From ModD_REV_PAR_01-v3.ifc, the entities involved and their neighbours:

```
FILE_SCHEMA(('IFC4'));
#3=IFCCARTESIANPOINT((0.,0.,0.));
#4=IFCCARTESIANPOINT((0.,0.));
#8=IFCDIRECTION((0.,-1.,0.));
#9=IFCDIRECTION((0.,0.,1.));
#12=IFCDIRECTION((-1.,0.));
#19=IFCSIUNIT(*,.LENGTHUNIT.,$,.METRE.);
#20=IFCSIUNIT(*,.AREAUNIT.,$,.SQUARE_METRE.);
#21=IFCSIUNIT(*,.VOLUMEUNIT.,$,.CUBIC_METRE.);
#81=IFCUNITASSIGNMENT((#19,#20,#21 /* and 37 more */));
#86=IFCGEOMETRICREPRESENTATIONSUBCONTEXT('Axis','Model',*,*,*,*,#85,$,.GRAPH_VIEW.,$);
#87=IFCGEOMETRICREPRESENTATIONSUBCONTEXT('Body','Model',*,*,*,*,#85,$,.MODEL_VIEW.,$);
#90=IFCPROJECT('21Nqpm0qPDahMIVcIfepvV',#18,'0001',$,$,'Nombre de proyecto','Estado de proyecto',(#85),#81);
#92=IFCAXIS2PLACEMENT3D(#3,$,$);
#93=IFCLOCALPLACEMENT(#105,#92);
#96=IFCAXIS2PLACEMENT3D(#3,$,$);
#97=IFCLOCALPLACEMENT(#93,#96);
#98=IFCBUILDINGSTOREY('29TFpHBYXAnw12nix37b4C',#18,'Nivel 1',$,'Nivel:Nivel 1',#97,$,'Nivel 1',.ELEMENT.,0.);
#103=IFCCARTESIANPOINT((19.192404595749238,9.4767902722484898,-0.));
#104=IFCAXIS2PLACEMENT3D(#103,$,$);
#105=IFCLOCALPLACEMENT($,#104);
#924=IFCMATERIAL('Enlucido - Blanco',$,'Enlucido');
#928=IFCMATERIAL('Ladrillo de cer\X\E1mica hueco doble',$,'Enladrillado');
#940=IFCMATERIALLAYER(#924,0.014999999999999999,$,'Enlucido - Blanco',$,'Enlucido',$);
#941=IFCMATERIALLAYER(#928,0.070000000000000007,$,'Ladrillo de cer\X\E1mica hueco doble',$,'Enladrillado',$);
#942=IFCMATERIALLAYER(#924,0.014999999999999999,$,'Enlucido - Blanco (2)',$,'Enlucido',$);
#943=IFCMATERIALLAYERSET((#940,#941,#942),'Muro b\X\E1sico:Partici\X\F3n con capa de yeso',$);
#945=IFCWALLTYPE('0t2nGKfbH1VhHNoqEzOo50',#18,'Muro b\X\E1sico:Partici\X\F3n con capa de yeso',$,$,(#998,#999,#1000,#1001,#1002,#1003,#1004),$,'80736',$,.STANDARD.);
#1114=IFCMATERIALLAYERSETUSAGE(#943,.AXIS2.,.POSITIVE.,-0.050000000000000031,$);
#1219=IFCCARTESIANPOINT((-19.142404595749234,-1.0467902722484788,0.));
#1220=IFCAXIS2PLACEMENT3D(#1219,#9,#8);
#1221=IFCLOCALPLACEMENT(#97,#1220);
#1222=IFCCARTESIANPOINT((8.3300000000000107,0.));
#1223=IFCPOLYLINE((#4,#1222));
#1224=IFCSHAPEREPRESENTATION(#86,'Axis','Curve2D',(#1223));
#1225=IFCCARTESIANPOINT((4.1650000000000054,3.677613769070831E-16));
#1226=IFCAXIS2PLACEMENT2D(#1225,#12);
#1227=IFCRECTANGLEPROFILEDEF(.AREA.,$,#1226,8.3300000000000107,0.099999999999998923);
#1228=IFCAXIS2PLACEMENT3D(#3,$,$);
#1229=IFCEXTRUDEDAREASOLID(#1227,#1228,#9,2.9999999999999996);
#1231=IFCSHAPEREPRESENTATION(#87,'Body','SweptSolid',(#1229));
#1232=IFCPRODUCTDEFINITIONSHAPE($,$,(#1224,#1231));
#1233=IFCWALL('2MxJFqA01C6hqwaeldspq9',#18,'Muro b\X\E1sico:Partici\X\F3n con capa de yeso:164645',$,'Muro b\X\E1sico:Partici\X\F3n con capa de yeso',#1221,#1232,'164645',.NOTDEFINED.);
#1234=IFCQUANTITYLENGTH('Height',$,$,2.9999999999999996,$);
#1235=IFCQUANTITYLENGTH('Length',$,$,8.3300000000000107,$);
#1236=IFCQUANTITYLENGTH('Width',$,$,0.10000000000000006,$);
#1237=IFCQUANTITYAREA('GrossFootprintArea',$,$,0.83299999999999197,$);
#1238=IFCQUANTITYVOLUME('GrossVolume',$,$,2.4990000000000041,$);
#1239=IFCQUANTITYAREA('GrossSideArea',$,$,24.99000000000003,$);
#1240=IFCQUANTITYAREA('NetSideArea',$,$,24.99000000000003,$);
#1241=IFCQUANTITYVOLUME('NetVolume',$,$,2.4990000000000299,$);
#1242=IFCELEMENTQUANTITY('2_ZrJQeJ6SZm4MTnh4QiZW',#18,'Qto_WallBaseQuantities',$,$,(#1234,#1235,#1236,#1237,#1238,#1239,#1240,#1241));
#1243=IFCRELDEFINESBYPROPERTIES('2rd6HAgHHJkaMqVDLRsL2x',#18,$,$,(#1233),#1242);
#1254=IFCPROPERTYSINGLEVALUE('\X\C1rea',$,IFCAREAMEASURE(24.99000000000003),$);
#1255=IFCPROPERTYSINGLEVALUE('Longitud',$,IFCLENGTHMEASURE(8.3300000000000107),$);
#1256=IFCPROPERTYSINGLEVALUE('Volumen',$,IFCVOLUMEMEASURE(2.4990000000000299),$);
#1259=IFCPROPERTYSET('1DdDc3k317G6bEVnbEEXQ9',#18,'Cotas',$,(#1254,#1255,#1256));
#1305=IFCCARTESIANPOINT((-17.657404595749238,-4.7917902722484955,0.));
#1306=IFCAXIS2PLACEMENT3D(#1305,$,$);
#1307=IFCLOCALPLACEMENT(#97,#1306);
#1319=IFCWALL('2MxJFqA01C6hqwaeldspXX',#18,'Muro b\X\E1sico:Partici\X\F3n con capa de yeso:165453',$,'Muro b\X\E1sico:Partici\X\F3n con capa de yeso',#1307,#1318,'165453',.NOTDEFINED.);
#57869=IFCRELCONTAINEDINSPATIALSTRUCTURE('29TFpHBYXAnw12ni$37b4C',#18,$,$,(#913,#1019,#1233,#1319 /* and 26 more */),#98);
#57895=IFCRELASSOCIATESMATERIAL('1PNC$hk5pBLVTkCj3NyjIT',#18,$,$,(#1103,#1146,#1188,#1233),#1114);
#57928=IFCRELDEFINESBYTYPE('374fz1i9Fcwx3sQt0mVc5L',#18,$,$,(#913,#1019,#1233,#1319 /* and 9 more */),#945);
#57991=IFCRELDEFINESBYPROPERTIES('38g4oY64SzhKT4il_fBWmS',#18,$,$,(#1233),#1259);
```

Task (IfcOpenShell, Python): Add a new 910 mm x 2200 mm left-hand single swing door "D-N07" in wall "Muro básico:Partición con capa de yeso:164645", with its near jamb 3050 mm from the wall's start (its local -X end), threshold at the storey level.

```python
import numpy as np
import ifcopenshell
import ifcopenshell.api.feature
import ifcopenshell.api.geometry
import ifcopenshell.api.pset
import ifcopenshell.api.root
import ifcopenshell.api.spatial
import ifcopenshell.geom
import ifcopenshell.util.element
import ifcopenshell.util.placement
import ifcopenshell.util.representation
import ifcopenshell.util.shape
import ifcopenshell.util.unit

model = ifcopenshell.open("ModD_REV_PAR_01-v3.ifc")
unit_scale = ifcopenshell.util.unit.calculate_unit_scale(model)
area_scale = ifcopenshell.util.unit.calculate_unit_scale(model, "AREAUNIT")
volume_scale = ifcopenshell.util.unit.calculate_unit_scale(model, "VOLUMEUNIT")
settings = ifcopenshell.geom.settings()


def volume(element):
    """Net volume in cubic metres, openings subtracted."""
    shape = ifcopenshell.geom.create_shape(settings, element)
    return ifcopenshell.util.shape.get_volume(shape.geometry)


wall = model.by_guid("2MxJFqA01C6hqwaeldspq9")
storey = ifcopenshell.util.element.get_container(wall, ifc_class="IfcBuildingStorey")
context = ifcopenshell.util.representation.get_context(model, "Model", "Body", "MODEL_VIEW")
before = volume(wall)

width, height, from_end, sill = 0.91, 2.2, 3.05, 0.0  # metres

# The wall runs along its own X axis, and the end named is its -X end.
wall_shape = ifcopenshell.geom.create_shape(settings, wall)
x, y, z = ifcopenshell.util.shape.get_vertices(wall_shape.geometry).T
start = x.min() + from_end
face, thickness = float(y.min()), float(y.max() - y.min())
wall_matrix = ifcopenshell.util.placement.get_local_placement(wall.ObjectPlacement)
level = ifcopenshell.util.placement.get_local_placement(storey.ObjectPlacement)[2, 3]


def in_wall(x, y):
    """Placement at x, y metres in the wall's axes, at sill height."""
    matrix = wall_matrix.copy()
    matrix[:, 3] = wall_matrix @ np.array([x / unit_scale, y / unit_scale, 0.0, 1.0])
    matrix[2, 3] = level + sill / unit_scale
    return matrix


# Opening: a box that overshoots both wall faces by 50 mm.
opening = ifcopenshell.api.root.create_entity(model, ifc_class="IfcOpeningElement", predefined_type="OPENING")
box = ifcopenshell.api.geometry.add_wall_representation(
    model, context=context, length=width, height=height, thickness=thickness + 0.1
)
ifcopenshell.api.geometry.assign_representation(model, product=opening, representation=box)
ifcopenshell.api.geometry.edit_object_placement(model, product=opening, matrix=in_wall(start, face - 0.05), is_si=False)
ifcopenshell.api.feature.add_feature(model, feature=opening, element=wall)

door = ifcopenshell.api.root.create_entity(model, ifc_class="IfcDoor", name="D-N07", predefined_type="DOOR")
door.OverallWidth, door.OverallHeight = width / unit_scale, height / unit_scale
door.OperationType = "SINGLE_SWING_LEFT"
body = ifcopenshell.api.geometry.add_door_representation(
    model,
    context=context,
    overall_width=door.OverallWidth,
    overall_height=door.OverallHeight,
    operation_type="SINGLE_SWING_LEFT",
    lining_properties={"LiningDepth": thickness / unit_scale, "ThresholdDepth": thickness / unit_scale},
)
ifcopenshell.api.geometry.assign_representation(model, product=door, representation=body)
ifcopenshell.api.spatial.assign_container(model, products=[door], relating_structure=storey)
ifcopenshell.api.feature.add_filling(model, opening=opening, element=door)

# The lining spans the wall, so the door starts at the wall face.
ifcopenshell.api.geometry.edit_object_placement(model, product=door, matrix=in_wall(start, face), is_si=False)

after = volume(wall)

# Update the wall's stored quantities.
qto = model.by_id(ifcopenshell.util.element.get_pset(wall, "Qto_WallBaseQuantities", should_inherit=False)["id"])
ifcopenshell.api.pset.edit_qto(model, qto=qto, properties={
    "NetSideArea": after / thickness / area_scale,
    "NetVolume": after / volume_scale,
})
pset = model.by_id(ifcopenshell.util.element.get_pset(wall, "Cotas", should_inherit=False)["id"])
ifcopenshell.api.pset.edit_pset(model, pset=pset, properties={
    "Área": model.create_entity("IfcAreaMeasure", after / thickness / area_scale),
    "Volumen": model.create_entity("IfcVolumeMeasure", after / volume_scale),
})

print(f"wall volume {before:.3f} -> {after:.3f} m3")

model.write("ModD_REV_PAR_01-v3-out.ifc")
```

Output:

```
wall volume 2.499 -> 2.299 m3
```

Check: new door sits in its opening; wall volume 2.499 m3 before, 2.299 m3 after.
